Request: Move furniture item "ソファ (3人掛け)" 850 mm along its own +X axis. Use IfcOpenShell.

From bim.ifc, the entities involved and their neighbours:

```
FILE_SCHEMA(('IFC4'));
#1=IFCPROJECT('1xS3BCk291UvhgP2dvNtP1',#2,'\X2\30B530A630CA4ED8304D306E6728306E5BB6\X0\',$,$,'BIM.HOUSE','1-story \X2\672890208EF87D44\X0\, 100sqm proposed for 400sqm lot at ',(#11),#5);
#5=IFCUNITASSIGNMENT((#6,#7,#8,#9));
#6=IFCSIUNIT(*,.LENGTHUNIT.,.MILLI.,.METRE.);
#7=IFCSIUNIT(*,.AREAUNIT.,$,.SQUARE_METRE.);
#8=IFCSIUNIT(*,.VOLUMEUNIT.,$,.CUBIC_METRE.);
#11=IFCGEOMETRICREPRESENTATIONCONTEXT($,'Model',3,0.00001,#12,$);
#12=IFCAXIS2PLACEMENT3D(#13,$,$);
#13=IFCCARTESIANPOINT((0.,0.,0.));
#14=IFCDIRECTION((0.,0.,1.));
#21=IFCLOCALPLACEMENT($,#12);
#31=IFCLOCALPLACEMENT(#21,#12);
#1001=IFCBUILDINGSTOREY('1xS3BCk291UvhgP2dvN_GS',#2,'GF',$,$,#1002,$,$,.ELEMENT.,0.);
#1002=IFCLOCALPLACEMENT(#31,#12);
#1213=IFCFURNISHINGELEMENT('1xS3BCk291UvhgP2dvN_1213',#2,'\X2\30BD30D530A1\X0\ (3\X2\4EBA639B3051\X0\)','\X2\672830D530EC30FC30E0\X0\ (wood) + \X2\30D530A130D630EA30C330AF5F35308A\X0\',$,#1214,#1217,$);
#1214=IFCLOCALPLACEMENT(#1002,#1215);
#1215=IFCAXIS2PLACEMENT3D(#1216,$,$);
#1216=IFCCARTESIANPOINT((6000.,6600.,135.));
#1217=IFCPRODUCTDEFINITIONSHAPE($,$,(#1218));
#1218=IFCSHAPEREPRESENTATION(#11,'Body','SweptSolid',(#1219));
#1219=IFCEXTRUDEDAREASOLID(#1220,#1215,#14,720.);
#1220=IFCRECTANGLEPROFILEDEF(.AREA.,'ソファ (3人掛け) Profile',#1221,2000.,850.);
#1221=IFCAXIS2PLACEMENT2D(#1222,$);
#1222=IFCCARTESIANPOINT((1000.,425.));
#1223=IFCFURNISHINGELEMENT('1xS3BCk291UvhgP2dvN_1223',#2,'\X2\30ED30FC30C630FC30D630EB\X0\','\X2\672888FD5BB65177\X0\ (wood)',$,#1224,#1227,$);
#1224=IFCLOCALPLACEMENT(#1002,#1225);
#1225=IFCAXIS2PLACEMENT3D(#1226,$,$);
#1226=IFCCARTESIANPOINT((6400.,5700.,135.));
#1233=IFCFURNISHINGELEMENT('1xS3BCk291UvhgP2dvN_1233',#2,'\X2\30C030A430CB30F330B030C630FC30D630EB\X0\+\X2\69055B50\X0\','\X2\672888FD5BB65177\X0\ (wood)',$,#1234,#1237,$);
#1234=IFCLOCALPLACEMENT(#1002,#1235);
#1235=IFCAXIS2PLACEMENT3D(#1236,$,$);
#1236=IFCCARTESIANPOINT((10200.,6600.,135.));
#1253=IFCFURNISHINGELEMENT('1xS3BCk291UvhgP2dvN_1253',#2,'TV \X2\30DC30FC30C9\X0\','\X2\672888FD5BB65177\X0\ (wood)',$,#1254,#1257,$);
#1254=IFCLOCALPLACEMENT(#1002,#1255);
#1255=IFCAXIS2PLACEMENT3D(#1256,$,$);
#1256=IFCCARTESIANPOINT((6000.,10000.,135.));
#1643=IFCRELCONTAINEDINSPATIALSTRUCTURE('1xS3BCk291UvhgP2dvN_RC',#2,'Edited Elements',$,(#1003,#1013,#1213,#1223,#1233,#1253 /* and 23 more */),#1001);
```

```python
import ifcopenshell
import ifcopenshell.api.geometry
import ifcopenshell.util.placement

model = ifcopenshell.open("bim.ifc")

item = model.by_guid("1xS3BCk291UvhgP2dvN_1213")
matrix = ifcopenshell.util.placement.get_local_placement(item.ObjectPlacement)
matrix[:3, 3] += matrix[:3, 0] * 850.0
ifcopenshell.api.geometry.edit_object_placement(model, product=item, matrix=matrix, is_si=False)

print(ifcopenshell.util.placement.get_local_placement(item.ObjectPlacement).round(3) + 0.0)

model.write("bim_updated.ifc")
```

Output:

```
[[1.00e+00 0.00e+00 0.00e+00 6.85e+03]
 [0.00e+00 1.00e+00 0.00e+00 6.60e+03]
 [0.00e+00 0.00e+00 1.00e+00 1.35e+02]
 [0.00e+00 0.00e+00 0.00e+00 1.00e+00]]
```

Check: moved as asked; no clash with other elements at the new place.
